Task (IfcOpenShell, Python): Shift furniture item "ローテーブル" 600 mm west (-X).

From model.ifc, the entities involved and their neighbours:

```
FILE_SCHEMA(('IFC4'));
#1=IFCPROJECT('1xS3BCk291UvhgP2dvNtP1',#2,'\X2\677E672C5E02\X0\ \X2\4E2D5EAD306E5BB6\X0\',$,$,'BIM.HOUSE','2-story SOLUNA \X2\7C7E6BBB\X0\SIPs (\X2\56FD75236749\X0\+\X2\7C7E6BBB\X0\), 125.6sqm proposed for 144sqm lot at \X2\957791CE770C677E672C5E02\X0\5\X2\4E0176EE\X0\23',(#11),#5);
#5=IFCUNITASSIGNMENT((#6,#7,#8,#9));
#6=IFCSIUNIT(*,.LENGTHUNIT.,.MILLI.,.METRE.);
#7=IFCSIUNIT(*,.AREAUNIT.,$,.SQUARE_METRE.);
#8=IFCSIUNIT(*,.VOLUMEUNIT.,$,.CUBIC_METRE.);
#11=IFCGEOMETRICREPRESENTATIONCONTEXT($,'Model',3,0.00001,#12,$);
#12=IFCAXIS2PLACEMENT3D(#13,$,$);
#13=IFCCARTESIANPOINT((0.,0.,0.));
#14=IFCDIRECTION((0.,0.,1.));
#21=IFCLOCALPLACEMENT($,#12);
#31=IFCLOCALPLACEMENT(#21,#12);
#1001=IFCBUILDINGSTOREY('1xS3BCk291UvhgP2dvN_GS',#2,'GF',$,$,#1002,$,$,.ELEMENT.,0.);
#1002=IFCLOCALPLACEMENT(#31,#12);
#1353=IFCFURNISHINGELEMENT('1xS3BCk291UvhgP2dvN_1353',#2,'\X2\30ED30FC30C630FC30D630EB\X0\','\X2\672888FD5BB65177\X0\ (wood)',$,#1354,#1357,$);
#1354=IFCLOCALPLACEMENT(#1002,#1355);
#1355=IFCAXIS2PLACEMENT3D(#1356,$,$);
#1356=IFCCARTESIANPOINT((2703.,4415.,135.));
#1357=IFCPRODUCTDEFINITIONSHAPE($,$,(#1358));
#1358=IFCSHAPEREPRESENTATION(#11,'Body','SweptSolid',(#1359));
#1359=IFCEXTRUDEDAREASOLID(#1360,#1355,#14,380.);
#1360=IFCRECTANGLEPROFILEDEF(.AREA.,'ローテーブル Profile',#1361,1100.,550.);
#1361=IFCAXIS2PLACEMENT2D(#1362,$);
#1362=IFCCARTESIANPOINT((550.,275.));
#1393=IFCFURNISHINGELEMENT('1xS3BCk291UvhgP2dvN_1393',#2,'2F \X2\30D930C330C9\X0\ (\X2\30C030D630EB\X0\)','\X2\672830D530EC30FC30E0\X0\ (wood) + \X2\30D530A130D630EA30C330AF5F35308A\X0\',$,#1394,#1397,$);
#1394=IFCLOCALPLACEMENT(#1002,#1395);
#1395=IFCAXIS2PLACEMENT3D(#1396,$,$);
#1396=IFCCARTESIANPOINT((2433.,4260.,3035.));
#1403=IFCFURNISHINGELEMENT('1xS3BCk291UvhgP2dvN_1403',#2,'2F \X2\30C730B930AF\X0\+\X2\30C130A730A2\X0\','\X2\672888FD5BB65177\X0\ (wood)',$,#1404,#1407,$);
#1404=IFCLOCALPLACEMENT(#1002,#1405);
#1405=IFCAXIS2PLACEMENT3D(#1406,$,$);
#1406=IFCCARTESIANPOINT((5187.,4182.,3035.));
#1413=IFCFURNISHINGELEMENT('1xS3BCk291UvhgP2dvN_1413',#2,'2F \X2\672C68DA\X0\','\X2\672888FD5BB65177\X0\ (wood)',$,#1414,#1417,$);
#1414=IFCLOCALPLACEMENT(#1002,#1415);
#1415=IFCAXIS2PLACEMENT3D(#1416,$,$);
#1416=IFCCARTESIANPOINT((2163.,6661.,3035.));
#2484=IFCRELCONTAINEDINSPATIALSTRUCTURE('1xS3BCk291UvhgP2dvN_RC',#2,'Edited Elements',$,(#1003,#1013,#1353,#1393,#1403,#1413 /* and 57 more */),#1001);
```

```python
import ifcopenshell
import ifcopenshell.api.geometry
import ifcopenshell.util.placement
import ifcopenshell.util.unit

model = ifcopenshell.open("model.ifc")
unit_scale = ifcopenshell.util.unit.calculate_unit_scale(model)

item = model.by_guid("1xS3BCk291UvhgP2dvN_1353")
matrix = ifcopenshell.util.placement.get_local_placement(item.ObjectPlacement)
matrix[0, 3] -= 0.6 / unit_scale
ifcopenshell.api.geometry.edit_object_placement(model, product=item, matrix=matrix, is_si=False)

print(ifcopenshell.util.placement.get_local_placement(item.ObjectPlacement).round(3) + 0.0)

model.write("model_rev.ifc")
```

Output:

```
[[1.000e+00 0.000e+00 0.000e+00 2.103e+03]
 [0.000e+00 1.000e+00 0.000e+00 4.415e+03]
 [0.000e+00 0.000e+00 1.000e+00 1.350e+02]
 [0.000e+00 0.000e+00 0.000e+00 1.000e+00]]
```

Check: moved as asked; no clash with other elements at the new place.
